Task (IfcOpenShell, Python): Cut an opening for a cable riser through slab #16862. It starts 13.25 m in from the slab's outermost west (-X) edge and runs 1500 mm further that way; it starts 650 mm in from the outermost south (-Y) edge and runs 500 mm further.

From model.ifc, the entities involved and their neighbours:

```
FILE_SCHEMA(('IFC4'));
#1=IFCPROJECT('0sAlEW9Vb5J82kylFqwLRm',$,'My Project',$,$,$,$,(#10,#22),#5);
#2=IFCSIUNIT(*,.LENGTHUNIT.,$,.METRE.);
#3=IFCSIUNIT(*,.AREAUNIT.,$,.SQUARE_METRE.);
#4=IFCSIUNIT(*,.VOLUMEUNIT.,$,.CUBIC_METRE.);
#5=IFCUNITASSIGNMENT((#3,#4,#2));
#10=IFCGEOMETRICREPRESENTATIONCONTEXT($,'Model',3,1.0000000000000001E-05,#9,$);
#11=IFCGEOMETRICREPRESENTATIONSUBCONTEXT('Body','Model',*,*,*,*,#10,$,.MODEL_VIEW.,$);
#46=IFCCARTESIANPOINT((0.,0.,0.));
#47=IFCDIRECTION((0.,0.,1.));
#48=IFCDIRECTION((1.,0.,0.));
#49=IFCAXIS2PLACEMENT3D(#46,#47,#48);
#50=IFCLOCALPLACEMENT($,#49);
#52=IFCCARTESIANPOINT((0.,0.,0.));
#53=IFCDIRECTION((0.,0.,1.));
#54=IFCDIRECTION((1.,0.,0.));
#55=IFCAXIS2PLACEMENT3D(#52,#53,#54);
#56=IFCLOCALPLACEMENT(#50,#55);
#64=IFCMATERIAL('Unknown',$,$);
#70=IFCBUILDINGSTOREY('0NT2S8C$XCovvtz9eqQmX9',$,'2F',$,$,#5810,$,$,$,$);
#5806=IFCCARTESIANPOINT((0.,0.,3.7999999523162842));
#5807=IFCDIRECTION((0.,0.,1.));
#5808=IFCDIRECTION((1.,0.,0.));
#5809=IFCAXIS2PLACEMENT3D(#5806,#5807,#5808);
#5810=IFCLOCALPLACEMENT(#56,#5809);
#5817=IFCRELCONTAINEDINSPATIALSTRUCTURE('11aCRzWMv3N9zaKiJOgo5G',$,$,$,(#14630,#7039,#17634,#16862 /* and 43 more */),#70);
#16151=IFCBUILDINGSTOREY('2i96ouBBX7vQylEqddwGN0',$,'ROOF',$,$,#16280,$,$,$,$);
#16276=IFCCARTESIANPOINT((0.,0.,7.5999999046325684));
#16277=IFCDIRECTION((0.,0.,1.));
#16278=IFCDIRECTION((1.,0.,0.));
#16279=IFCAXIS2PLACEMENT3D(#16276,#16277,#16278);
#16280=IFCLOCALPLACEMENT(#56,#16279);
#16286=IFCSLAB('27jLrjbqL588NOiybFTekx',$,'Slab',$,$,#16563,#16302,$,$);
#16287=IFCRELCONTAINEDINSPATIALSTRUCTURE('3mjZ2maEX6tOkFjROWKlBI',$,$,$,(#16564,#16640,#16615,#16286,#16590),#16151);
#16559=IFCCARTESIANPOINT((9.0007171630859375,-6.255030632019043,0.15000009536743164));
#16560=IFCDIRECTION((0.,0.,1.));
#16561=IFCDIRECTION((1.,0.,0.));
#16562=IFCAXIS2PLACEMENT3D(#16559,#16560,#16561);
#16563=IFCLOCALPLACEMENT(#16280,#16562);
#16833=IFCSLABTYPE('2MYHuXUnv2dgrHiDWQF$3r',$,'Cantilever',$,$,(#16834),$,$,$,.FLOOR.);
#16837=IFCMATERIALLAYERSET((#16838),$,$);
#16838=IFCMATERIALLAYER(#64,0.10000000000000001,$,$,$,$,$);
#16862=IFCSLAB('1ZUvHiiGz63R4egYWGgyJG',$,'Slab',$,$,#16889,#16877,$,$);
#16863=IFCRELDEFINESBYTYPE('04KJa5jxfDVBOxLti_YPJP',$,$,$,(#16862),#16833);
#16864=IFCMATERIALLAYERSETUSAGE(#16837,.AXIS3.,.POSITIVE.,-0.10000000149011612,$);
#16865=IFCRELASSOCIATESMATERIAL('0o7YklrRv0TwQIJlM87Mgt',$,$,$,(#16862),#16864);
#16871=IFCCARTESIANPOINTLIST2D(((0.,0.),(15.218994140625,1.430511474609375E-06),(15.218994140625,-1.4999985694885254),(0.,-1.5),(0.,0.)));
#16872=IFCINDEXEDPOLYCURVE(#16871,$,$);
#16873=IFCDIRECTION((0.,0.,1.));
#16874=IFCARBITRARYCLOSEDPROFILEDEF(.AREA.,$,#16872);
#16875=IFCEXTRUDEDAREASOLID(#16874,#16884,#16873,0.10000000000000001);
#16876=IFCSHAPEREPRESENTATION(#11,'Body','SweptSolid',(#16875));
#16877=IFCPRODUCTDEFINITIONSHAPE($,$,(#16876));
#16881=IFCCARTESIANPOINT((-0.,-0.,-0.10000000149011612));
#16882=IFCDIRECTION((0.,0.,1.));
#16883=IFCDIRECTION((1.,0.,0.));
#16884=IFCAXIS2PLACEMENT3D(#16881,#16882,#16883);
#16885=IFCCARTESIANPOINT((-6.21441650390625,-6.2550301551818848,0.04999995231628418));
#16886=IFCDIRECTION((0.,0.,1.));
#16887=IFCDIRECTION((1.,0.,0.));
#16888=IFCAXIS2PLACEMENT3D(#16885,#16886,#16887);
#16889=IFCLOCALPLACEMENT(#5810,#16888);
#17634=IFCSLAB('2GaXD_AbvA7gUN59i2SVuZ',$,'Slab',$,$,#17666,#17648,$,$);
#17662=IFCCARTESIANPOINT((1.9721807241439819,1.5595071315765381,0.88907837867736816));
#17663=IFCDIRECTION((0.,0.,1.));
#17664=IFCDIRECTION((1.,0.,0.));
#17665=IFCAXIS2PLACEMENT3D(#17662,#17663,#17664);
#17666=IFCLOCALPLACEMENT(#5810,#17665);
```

```python
import numpy as np
import ifcopenshell
import ifcopenshell.api.feature
import ifcopenshell.api.geometry
import ifcopenshell.api.root
import ifcopenshell.geom
import ifcopenshell.util.placement
import ifcopenshell.util.representation
import ifcopenshell.util.shape
import ifcopenshell.util.unit

model = ifcopenshell.open("model.ifc")
unit_scale = ifcopenshell.util.unit.calculate_unit_scale(model)
settings = ifcopenshell.geom.settings()


def volume(element):
    """Net volume in cubic metres, openings subtracted."""
    shape = ifcopenshell.geom.create_shape(settings, element)
    return ifcopenshell.util.shape.get_volume(shape.geometry)


slab = model.by_guid("1ZUvHiiGz63R4egYWGgyJG")
before = volume(slab)

# Extent in the slab's own axes, in metres. The edges named are its -X and -Y sides.
slab_shape = ifcopenshell.geom.create_shape(settings, slab)
vertices = ifcopenshell.util.shape.get_vertices(slab_shape.geometry)
x_min, y_min, bottom = vertices.min(axis=0)
top = vertices[:, 2].max()

opening = ifcopenshell.api.root.create_entity(model, ifc_class="IfcOpeningElement", name="Cable riser opening", predefined_type="OPENING")
context = ifcopenshell.util.representation.get_context(model, "Model", "Body", "MODEL_VIEW")
width, depth = 1.5, 0.5
outline = [(0.0, 0.0), (width, 0.0), (width, depth), (0.0, depth), (0.0, 0.0)]
# Overshoot both faces by 50 mm so the cut is clean.
shape = ifcopenshell.api.geometry.add_slab_representation(
    model, context=context, depth=top - bottom + 0.1, polyline=outline
)
ifcopenshell.api.geometry.assign_representation(model, product=opening, representation=shape)

matrix = ifcopenshell.util.placement.get_local_placement(slab.ObjectPlacement)
matrix[:, 3] = matrix @ np.append(np.array([x_min + 13.25, y_min + 0.65, bottom - 0.05]) / unit_scale, 1.0)
ifcopenshell.api.geometry.edit_object_placement(model, product=opening, matrix=matrix, is_si=False)
ifcopenshell.api.feature.add_feature(model, feature=opening, element=slab)

after = volume(slab)

print(f"slab volume {before:.3f} -> {after:.3f} m3")

model.write("model-out.ifc")
```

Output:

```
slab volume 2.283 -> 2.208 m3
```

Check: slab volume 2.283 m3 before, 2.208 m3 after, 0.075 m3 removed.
